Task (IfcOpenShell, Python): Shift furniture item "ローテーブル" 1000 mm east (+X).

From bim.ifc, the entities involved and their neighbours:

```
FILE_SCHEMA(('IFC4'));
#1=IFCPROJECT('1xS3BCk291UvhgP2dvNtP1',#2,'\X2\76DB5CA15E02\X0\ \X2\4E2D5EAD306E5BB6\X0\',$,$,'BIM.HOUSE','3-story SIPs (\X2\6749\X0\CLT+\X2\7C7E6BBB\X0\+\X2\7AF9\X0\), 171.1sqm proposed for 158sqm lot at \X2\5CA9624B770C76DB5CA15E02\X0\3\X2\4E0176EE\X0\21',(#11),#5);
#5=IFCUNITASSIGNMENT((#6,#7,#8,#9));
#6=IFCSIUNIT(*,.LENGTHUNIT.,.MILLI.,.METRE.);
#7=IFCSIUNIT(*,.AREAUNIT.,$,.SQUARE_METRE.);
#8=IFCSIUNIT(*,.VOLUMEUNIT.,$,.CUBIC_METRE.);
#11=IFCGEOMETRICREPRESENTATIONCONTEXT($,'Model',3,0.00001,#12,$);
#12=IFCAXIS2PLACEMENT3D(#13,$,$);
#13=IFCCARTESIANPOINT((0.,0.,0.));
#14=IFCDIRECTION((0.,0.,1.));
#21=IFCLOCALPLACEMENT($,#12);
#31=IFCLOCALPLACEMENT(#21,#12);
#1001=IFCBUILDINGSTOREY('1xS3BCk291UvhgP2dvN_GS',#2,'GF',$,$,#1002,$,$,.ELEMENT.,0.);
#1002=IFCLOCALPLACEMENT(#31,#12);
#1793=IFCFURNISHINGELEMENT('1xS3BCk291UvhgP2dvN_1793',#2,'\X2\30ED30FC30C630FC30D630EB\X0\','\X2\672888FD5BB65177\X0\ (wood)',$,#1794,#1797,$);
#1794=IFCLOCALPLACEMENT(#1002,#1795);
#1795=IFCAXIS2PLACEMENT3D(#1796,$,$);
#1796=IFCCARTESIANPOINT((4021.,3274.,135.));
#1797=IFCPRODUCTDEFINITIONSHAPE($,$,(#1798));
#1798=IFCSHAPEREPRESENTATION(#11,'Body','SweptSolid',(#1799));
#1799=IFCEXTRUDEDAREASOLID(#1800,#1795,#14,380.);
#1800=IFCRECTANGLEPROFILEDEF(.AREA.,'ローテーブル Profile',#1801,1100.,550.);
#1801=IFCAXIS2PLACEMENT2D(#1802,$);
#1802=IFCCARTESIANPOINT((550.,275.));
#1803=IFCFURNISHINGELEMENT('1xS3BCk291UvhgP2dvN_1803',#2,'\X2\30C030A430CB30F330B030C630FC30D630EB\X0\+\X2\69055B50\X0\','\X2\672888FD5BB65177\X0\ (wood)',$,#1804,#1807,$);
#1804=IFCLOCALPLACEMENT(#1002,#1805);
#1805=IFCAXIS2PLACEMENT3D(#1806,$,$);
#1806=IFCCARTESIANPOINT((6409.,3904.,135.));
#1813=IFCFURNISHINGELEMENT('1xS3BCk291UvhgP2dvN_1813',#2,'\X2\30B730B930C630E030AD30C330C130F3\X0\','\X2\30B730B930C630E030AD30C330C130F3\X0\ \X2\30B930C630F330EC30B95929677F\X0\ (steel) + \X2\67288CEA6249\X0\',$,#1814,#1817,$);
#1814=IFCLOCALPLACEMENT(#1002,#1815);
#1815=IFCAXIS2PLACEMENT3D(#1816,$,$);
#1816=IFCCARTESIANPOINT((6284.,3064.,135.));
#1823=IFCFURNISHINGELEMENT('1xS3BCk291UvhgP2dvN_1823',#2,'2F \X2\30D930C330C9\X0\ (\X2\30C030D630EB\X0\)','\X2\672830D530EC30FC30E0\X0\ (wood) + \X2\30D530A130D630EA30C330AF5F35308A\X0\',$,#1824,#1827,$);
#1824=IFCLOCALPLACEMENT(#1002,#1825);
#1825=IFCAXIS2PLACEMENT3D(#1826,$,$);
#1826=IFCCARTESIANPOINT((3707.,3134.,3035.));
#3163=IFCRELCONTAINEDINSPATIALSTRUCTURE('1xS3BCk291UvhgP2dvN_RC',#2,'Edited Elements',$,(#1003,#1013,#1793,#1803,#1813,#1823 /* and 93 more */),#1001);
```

```python
import ifcopenshell
import ifcopenshell.api.geometry
import ifcopenshell.util.placement
import ifcopenshell.util.unit

model = ifcopenshell.open("bim.ifc")
unit_scale = ifcopenshell.util.unit.calculate_unit_scale(model)

item = model.by_id(1793)
matrix = ifcopenshell.util.placement.get_local_placement(item.ObjectPlacement)
matrix[0, 3] += 1 / unit_scale
ifcopenshell.api.geometry.edit_object_placement(model, product=item, matrix=matrix, is_si=False)

print(ifcopenshell.util.placement.get_local_placement(item.ObjectPlacement).round(3) + 0.0)

model.write("bim-out.ifc")
```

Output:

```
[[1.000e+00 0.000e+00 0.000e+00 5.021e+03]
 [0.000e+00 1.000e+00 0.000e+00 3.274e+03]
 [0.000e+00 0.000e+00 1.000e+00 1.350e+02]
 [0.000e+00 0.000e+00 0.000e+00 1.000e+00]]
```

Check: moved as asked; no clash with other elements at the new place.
